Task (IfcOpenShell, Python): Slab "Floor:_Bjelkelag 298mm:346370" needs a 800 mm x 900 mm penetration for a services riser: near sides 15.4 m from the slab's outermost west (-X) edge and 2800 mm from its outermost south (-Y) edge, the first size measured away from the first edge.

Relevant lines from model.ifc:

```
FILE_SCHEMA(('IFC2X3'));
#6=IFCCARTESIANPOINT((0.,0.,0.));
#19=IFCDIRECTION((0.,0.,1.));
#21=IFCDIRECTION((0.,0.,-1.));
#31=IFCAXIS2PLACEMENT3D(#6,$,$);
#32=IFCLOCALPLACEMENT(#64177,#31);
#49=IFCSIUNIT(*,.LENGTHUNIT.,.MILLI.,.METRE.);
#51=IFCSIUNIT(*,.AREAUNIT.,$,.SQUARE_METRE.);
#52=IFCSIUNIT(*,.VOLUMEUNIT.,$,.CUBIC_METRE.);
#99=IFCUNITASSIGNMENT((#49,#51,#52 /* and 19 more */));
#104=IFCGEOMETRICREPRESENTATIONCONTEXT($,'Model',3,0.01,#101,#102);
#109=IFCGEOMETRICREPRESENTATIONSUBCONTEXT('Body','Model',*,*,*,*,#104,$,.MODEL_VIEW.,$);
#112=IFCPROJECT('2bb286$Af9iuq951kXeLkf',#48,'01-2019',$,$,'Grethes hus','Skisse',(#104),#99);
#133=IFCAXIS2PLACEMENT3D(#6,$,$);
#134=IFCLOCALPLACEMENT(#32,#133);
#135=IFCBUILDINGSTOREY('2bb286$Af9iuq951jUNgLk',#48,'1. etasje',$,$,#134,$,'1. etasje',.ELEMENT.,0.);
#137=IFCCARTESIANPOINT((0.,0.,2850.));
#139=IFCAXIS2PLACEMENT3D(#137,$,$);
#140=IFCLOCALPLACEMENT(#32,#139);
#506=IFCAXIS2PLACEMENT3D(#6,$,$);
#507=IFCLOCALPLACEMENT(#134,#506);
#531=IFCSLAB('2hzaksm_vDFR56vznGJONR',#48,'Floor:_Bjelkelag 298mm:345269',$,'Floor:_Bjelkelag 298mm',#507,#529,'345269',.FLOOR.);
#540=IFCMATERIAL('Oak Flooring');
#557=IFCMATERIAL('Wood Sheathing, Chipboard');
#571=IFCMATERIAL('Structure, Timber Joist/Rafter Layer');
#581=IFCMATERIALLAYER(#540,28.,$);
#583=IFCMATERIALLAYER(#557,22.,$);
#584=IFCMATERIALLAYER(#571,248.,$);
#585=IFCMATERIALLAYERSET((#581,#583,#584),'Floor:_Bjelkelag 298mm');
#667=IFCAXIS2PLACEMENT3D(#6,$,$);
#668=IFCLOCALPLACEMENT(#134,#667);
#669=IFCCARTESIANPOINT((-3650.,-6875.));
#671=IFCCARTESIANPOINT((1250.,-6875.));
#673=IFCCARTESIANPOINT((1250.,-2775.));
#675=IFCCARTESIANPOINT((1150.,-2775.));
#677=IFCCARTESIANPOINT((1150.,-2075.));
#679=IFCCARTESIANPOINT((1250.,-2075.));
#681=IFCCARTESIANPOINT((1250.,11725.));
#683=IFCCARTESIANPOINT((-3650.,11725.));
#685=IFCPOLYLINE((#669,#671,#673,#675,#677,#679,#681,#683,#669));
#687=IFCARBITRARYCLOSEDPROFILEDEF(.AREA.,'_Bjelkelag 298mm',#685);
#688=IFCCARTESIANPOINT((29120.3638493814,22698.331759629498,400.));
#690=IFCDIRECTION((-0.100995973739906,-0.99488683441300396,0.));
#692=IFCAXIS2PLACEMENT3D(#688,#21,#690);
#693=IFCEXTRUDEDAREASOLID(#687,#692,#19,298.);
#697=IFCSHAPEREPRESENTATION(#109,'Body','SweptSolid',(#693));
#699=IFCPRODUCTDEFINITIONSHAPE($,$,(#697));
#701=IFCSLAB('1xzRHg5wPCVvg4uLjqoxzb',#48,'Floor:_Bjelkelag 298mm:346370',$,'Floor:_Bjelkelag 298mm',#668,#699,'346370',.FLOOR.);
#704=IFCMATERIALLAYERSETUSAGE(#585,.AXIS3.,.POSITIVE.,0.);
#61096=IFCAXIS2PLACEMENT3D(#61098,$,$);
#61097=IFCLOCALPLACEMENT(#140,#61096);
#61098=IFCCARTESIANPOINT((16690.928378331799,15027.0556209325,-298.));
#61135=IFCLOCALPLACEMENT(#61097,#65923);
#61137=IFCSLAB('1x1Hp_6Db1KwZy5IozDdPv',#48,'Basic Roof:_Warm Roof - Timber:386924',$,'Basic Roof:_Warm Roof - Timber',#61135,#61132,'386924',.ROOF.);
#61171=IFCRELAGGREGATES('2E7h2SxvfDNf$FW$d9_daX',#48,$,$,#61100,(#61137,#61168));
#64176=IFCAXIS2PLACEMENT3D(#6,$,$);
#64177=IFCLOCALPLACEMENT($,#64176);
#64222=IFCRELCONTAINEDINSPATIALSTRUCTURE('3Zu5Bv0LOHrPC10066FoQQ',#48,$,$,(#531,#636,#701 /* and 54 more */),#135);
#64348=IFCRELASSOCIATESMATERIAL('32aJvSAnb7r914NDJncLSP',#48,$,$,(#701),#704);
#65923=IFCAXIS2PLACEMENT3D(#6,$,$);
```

```python
import numpy as np
import ifcopenshell
import ifcopenshell.api.feature
import ifcopenshell.api.geometry
import ifcopenshell.api.root
import ifcopenshell.geom
import ifcopenshell.util.placement
import ifcopenshell.util.representation
import ifcopenshell.util.shape
import ifcopenshell.util.unit

model = ifcopenshell.open("model.ifc")
unit_scale = ifcopenshell.util.unit.calculate_unit_scale(model)
settings = ifcopenshell.geom.settings()


def volume(element):
    """Net volume in cubic metres, openings subtracted."""
    shape = ifcopenshell.geom.create_shape(settings, element)
    return ifcopenshell.util.shape.get_volume(shape.geometry)


slab = model.by_id(701)
before = volume(slab)

# Extent in the slab's own axes, in metres. The edges named are its -X and -Y sides.
slab_shape = ifcopenshell.geom.create_shape(settings, slab)
vertices = ifcopenshell.util.shape.get_vertices(slab_shape.geometry)
x_min, y_min, bottom = vertices.min(axis=0)
top = vertices[:, 2].max()

opening = ifcopenshell.api.root.create_entity(model, ifc_class="IfcOpeningElement", name="Services riser opening")
context = ifcopenshell.util.representation.get_context(model, "Model", "Body", "MODEL_VIEW")
width, depth = 0.8, 0.9
outline = [(0.0, 0.0), (width, 0.0), (width, depth), (0.0, depth), (0.0, 0.0)]
# Overshoot both faces by 50 mm so the cut is clean.
shape = ifcopenshell.api.geometry.add_slab_representation(
    model, context=context, depth=top - bottom + 0.1, polyline=outline
)
ifcopenshell.api.geometry.assign_representation(model, product=opening, representation=shape)

matrix = ifcopenshell.util.placement.get_local_placement(slab.ObjectPlacement)
matrix[:, 3] = matrix @ np.append(np.array([x_min + 15.4, y_min + 2.8, bottom - 0.05]) / unit_scale, 1.0)
ifcopenshell.api.geometry.edit_object_placement(model, product=opening, matrix=matrix, is_si=False)
ifcopenshell.api.feature.add_feature(model, feature=opening, element=slab)

after = volume(slab)

print(f"slab volume {before:.3f} -> {after:.3f} m3")

model.write("model-out.ifc")
```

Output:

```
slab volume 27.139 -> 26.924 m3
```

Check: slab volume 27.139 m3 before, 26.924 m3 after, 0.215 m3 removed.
